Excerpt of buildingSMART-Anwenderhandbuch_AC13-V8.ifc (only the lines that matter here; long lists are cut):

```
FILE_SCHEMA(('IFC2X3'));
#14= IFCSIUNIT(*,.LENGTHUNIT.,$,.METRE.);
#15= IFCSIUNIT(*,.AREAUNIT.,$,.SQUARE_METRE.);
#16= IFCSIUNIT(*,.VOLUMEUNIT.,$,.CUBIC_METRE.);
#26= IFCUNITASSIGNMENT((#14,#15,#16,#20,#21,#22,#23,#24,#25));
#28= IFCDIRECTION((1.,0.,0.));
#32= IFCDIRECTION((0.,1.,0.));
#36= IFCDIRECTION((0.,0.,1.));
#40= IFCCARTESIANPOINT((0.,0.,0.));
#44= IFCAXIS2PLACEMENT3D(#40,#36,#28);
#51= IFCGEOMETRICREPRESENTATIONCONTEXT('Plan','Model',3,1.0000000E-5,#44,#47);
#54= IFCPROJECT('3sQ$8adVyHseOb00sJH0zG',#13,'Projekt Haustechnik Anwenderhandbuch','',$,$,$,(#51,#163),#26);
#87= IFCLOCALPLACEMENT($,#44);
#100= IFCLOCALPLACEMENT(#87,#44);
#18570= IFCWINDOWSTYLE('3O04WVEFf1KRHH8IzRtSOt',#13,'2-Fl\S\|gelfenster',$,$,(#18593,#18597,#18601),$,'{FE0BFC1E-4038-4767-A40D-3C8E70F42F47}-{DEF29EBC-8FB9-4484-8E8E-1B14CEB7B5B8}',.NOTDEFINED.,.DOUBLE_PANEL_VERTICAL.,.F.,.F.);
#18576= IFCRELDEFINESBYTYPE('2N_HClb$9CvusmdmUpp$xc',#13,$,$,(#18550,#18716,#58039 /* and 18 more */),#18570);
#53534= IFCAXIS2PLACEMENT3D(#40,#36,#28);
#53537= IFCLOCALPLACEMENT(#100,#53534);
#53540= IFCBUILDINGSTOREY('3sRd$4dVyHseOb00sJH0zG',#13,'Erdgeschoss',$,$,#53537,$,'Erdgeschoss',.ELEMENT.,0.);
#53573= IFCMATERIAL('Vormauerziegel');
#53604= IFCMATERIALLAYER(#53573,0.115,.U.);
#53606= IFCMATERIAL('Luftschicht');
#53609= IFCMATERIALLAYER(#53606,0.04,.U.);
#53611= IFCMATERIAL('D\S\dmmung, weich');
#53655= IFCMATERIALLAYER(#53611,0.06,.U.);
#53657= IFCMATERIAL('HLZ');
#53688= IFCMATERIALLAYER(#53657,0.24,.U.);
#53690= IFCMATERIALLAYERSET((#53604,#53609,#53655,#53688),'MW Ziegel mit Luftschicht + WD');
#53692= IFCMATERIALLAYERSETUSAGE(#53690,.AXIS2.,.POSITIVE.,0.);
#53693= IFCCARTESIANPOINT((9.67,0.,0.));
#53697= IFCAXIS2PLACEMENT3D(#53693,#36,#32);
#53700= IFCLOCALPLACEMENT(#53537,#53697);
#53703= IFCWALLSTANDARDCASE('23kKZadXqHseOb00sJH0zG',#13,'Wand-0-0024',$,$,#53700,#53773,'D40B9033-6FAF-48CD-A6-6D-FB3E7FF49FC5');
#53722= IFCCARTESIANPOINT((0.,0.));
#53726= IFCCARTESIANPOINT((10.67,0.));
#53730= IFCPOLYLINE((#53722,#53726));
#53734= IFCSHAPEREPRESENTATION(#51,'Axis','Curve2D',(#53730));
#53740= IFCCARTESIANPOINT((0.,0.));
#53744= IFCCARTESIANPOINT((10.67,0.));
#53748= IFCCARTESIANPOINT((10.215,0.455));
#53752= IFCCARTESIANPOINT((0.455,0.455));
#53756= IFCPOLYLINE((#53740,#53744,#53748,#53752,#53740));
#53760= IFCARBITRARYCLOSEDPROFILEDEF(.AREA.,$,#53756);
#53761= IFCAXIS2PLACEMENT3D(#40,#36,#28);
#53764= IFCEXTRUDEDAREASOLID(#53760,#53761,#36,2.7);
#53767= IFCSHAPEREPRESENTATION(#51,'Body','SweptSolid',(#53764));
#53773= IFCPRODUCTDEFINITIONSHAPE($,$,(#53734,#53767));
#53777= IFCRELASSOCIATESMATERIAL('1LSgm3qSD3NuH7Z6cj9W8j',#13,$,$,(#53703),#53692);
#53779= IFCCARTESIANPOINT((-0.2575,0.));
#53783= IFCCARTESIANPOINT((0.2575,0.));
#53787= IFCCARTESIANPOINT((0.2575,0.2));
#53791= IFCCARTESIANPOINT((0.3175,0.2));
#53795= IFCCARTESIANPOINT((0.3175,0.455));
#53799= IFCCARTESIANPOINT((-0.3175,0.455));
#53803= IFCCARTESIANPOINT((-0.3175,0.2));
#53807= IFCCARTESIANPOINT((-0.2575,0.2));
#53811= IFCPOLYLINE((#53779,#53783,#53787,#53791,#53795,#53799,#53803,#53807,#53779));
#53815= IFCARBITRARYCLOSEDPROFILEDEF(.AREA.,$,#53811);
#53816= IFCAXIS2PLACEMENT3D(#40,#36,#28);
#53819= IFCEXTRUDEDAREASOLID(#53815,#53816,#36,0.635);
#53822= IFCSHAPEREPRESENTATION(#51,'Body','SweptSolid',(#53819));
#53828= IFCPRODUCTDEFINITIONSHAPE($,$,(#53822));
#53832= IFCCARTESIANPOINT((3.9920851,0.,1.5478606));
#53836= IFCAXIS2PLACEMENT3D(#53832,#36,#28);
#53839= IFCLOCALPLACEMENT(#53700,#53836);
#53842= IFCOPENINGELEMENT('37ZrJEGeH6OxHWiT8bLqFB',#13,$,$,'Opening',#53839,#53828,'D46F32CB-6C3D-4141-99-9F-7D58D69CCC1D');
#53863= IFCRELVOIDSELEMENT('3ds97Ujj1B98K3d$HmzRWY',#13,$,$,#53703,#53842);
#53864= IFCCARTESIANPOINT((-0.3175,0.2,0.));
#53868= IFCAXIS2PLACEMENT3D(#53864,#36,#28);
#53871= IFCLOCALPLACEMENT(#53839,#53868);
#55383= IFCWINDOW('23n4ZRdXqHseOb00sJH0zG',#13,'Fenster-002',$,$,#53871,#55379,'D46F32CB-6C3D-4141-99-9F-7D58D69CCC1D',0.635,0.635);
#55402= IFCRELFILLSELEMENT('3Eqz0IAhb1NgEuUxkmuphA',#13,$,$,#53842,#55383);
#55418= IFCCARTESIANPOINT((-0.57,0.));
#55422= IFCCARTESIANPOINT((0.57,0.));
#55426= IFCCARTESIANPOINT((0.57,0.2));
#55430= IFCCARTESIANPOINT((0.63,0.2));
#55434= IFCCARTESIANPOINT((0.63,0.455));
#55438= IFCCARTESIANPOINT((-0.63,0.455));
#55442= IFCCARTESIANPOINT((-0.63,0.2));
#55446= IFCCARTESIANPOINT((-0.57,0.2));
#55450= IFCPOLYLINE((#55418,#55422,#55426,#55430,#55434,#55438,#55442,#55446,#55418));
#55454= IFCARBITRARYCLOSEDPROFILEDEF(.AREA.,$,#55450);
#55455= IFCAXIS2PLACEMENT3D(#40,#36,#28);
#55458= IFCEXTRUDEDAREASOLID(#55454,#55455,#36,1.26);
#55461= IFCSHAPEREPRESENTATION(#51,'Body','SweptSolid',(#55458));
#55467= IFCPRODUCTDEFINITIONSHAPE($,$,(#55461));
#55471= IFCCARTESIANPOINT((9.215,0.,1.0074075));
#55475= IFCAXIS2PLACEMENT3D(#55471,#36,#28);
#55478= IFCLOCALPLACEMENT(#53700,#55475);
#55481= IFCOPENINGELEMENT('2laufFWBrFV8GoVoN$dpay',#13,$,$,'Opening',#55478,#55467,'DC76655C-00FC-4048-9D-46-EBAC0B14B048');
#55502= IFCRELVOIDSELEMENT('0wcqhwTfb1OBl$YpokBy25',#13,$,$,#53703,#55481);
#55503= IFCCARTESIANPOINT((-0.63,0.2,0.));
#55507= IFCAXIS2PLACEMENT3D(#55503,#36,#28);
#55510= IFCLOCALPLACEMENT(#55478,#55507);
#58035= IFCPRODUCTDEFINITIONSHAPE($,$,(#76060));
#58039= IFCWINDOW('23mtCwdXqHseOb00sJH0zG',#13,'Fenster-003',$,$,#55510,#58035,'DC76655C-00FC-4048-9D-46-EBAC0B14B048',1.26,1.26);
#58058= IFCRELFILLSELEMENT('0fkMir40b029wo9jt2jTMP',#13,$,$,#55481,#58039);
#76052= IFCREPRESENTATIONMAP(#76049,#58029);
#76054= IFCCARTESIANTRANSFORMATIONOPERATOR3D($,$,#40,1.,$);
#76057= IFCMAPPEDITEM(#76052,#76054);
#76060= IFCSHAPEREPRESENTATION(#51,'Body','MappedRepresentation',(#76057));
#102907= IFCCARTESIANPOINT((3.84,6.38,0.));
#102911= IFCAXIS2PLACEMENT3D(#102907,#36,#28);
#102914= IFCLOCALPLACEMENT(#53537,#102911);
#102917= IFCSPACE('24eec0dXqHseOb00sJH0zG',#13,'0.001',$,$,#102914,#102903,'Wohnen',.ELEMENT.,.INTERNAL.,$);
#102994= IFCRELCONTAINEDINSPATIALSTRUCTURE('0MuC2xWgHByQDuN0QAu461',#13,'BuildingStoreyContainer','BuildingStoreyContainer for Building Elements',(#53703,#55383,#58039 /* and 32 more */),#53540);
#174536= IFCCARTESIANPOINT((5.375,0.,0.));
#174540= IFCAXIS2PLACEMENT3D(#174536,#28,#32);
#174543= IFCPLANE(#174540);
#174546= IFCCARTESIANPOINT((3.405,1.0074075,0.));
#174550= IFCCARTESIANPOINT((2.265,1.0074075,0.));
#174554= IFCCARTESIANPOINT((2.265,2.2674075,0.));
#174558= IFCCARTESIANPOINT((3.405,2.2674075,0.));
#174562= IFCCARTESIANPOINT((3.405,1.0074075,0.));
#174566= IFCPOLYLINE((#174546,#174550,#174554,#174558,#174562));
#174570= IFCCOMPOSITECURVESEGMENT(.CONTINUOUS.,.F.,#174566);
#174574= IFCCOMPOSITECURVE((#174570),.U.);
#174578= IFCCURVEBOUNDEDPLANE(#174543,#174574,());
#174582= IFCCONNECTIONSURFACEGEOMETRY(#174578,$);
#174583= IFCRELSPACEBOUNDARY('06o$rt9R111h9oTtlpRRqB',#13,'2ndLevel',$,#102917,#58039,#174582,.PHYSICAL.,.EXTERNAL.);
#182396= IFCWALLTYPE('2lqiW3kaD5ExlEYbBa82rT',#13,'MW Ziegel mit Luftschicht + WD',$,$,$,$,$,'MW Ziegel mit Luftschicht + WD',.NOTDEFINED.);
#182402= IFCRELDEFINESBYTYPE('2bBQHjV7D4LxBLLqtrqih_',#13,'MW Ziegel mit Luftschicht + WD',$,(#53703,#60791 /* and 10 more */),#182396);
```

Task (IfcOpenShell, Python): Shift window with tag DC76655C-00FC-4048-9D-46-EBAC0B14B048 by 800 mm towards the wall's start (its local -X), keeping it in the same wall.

```python
import numpy as np
import ifcopenshell
import ifcopenshell.api.geometry
import ifcopenshell.util.placement
import ifcopenshell.util.unit

model = ifcopenshell.open("buildingSMART-Anwenderhandbuch_AC13-V8.ifc")
unit_scale = ifcopenshell.util.unit.calculate_unit_scale(model)

window = model.by_id(58039)
opening = window.FillsVoids[0].RelatingOpeningElement
wall = opening.VoidsElements[0].RelatingBuildingElement

wall_matrix = ifcopenshell.util.placement.get_local_placement(wall.ObjectPlacement)
shift = wall_matrix[:3, 0] * -0.8 / unit_scale
before = ifcopenshell.util.placement.get_local_placement(window.ObjectPlacement)[:3, 3].copy()

# The window is placed relative to its opening, so it follows when the opening moves.
matrix = ifcopenshell.util.placement.get_local_placement(opening.ObjectPlacement)
matrix[:3, 3] += shift
ifcopenshell.api.geometry.edit_object_placement(
    model, product=opening, matrix=matrix, is_si=False, should_transform_children=True
)

# Space boundary surfaces are stored in each space's coordinates; move them too.
for rel in window.ProvidesBoundaries:
    if not rel.ConnectionGeometry:
        continue
    surface = rel.ConnectionGeometry.SurfaceOnRelatingElement.BasisSurface
    space_matrix = ifcopenshell.util.placement.get_local_placement(rel.RelatingSpace.ObjectPlacement)
    point = np.array(surface.Position.Location.Coordinates) + space_matrix[:3, :3].T @ shift
    surface.Position = model.createIfcAxis2Placement3D(
        model.createIfcCartesianPoint(point.tolist()), surface.Position.Axis, surface.Position.RefDirection
    )

after = ifcopenshell.util.placement.get_local_placement(window.ObjectPlacement)[:3, 3]
print("window moved by", (after - before).round(3) + 0.0)

model.write("buildingSMART-Anwenderhandbuch_AC13-V8_updated.ifc")
```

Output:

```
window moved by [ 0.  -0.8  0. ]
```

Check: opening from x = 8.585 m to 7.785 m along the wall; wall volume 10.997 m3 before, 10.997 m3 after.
